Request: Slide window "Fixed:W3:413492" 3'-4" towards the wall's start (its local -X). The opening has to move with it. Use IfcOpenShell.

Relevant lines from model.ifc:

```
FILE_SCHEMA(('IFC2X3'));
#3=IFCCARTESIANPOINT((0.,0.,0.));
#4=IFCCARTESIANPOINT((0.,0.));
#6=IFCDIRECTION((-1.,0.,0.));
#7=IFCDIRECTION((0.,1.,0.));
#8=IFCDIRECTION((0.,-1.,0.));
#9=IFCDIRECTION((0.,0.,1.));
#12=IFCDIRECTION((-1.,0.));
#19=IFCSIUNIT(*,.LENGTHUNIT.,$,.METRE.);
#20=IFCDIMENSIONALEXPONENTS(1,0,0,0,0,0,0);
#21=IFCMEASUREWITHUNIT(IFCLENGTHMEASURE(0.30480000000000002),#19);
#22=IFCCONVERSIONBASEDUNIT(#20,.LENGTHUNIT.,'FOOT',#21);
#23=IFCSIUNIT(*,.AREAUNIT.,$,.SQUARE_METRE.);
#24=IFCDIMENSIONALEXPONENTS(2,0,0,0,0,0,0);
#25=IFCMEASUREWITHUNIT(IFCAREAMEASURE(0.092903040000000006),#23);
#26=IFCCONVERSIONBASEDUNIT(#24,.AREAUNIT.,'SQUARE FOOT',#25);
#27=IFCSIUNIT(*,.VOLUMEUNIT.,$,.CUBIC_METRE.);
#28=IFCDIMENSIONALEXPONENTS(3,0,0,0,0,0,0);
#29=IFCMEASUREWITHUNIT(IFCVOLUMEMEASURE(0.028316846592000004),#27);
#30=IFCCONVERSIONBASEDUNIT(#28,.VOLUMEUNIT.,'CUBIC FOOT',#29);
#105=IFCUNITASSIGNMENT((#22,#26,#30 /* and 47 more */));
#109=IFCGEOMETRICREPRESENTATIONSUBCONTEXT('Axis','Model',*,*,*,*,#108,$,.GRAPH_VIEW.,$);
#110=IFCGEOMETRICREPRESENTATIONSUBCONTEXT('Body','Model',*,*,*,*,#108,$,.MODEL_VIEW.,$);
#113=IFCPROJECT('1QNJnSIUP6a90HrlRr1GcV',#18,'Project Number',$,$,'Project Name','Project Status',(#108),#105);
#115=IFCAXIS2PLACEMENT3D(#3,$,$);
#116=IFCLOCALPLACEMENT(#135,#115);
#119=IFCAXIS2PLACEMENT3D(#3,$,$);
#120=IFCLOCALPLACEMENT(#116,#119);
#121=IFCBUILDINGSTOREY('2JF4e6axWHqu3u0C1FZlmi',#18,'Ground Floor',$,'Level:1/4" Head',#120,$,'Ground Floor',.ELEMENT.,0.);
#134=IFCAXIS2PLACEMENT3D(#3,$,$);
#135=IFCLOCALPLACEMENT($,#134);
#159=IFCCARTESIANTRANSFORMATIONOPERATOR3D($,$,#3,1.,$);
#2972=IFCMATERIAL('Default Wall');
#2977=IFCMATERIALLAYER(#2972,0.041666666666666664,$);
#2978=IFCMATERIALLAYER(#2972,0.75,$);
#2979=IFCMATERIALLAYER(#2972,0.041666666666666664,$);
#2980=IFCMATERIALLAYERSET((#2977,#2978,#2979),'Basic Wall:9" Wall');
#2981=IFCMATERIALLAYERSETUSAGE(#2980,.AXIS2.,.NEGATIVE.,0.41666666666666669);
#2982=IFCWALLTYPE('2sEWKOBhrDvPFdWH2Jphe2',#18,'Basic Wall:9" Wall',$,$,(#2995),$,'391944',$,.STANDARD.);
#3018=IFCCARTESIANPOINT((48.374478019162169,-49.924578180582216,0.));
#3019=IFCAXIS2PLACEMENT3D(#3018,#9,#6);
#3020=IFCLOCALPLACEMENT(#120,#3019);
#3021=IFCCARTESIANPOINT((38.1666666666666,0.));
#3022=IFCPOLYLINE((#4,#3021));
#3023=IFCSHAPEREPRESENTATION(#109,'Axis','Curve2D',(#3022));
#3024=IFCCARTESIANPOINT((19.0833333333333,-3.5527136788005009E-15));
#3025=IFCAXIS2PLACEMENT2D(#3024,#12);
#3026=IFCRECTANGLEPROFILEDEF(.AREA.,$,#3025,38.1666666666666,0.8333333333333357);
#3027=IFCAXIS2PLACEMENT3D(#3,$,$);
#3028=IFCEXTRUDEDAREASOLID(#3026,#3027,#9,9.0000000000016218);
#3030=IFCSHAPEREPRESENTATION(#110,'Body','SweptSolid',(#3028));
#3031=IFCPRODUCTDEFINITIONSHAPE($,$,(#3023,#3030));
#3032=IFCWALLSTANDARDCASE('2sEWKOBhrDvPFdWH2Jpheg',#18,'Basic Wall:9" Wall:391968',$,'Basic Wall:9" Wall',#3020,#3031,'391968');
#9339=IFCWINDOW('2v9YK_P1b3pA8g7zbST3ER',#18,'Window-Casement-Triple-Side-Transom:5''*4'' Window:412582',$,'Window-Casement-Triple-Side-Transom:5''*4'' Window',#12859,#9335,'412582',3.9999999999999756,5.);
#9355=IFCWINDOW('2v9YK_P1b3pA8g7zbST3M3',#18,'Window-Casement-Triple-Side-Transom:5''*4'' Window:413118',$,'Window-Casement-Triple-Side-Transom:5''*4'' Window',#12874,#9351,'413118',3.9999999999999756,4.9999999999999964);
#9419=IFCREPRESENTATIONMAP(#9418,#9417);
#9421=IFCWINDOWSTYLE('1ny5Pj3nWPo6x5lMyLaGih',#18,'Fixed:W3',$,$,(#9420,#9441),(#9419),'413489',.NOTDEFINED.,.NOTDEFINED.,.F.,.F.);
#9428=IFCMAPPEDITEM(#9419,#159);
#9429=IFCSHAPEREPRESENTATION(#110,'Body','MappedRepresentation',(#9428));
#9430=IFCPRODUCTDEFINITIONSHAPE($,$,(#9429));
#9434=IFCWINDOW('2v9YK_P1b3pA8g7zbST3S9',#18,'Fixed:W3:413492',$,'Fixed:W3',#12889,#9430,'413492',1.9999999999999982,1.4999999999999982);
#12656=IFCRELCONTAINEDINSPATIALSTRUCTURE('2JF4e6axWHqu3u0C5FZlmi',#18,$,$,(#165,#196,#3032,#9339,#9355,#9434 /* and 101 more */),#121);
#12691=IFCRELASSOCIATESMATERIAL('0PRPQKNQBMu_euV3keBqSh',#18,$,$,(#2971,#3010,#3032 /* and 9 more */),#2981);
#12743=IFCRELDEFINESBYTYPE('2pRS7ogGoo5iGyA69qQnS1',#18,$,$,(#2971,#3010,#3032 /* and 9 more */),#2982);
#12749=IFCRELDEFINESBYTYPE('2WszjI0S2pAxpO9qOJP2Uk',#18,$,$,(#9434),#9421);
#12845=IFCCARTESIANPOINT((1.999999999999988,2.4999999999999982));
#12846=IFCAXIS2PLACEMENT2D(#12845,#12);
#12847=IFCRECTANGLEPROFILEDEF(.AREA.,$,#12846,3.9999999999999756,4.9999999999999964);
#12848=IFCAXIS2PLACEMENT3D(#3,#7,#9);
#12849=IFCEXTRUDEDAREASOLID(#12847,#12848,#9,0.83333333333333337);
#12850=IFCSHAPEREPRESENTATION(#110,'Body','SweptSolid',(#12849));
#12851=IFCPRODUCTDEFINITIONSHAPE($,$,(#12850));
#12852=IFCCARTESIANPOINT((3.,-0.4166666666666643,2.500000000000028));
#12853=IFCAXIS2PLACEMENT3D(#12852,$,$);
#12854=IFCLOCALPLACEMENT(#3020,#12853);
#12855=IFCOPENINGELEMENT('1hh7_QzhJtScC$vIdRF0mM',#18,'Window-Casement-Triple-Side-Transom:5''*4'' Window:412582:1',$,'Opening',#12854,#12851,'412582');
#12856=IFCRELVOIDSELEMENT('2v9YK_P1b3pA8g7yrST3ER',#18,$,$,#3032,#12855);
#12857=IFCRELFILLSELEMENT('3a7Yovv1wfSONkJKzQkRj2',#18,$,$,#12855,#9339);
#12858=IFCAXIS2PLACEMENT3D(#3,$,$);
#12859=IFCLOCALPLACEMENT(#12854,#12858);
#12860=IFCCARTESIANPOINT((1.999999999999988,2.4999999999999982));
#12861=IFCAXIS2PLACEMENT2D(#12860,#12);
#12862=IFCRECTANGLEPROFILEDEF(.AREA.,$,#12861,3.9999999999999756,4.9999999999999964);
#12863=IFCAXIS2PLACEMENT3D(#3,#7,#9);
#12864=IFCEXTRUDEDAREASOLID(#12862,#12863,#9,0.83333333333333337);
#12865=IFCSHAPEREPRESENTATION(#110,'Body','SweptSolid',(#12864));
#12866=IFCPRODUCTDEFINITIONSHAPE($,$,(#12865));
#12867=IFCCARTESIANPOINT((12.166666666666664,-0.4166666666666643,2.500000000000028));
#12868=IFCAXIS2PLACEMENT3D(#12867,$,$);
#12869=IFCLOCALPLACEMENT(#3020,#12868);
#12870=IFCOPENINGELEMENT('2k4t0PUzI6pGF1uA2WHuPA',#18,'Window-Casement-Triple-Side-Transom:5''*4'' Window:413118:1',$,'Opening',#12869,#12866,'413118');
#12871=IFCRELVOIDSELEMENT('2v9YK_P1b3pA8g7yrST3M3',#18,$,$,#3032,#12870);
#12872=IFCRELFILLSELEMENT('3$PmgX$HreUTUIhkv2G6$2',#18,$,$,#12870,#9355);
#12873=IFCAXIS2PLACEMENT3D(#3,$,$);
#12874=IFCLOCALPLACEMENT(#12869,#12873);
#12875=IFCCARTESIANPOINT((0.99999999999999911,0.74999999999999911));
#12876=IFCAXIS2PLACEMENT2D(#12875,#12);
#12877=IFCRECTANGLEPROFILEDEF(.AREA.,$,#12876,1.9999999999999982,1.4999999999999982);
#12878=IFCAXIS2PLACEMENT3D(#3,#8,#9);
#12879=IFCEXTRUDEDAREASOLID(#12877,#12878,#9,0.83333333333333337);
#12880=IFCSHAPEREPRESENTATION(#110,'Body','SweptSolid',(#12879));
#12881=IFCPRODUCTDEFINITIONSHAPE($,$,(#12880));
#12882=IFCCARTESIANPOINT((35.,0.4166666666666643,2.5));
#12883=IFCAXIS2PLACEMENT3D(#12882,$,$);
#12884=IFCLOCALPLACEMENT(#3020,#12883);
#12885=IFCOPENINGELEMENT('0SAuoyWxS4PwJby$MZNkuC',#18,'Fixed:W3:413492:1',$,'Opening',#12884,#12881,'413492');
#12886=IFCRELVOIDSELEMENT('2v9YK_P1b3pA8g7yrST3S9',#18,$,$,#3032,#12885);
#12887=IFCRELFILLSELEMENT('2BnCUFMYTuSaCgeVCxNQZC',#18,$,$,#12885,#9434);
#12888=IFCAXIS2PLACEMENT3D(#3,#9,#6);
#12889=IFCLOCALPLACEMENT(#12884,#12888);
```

```python
import ifcopenshell
import ifcopenshell.api.geometry
import ifcopenshell.util.placement
import ifcopenshell.util.unit

model = ifcopenshell.open("model.ifc")
unit_scale = ifcopenshell.util.unit.calculate_unit_scale(model)

window = model.by_id(9434)
opening = window.FillsVoids[0].RelatingOpeningElement
wall = opening.VoidsElements[0].RelatingBuildingElement

wall_matrix = ifcopenshell.util.placement.get_local_placement(wall.ObjectPlacement)
shift = wall_matrix[:3, 0] * -40 * 0.0254 / unit_scale
before = ifcopenshell.util.placement.get_local_placement(window.ObjectPlacement)[:3, 3].copy()

# The window is placed relative to its opening, so it follows when the opening moves.
matrix = ifcopenshell.util.placement.get_local_placement(opening.ObjectPlacement)
matrix[:3, 3] += shift
ifcopenshell.api.geometry.edit_object_placement(
    model, product=opening, matrix=matrix, is_si=False, should_transform_children=True
)

after = ifcopenshell.util.placement.get_local_placement(window.ObjectPlacement)[:3, 3]
print("window moved by", (after - before).round(3) + 0.0)

model.write("model-out.ifc")
```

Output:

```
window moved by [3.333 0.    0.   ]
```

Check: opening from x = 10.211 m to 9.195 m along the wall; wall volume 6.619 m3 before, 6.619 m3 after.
